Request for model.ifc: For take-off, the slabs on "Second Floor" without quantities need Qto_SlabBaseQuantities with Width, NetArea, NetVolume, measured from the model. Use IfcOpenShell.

First a look at what the model holds.

```python
import ifcopenshell
import ifcopenshell.util.element
import ifcopenshell.util.unit

model = ifcopenshell.open("model.ifc")
print(model.schema)
for unit_type in ("LENGTHUNIT", "AREAUNIT", "VOLUMEUNIT"):
    print(unit_type, ifcopenshell.util.unit.calculate_unit_scale(model, unit_type))
storey = next(s for s in model.by_type("IfcBuildingStorey") if s.Name == "Second Floor")
slabs = [e for e in ifcopenshell.util.element.get_decomposition(storey) if e.is_a("IfcSlab")]
for e in sorted(slabs, key=lambda e: e.id()):
    print(e.id(), e.is_a(), e.Name, list(ifcopenshell.util.element.get_psets(e, qtos_only=True)), sep=" | ")
```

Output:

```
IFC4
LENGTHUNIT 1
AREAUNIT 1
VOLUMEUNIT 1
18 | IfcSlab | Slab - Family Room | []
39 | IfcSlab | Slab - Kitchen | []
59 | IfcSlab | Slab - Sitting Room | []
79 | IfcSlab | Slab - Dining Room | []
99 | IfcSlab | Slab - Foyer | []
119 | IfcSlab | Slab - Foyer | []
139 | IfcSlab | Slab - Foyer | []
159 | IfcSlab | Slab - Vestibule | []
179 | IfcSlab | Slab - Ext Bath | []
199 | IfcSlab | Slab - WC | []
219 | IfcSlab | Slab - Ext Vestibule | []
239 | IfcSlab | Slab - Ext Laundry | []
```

```python
import ifcopenshell
import ifcopenshell.api.pset
import ifcopenshell.geom
import ifcopenshell.util.element
import ifcopenshell.util.shape
import ifcopenshell.util.unit

model = ifcopenshell.open("model.ifc")
unit_scale = ifcopenshell.util.unit.calculate_unit_scale(model)
area_scale = ifcopenshell.util.unit.calculate_unit_scale(model, "AREAUNIT")
volume_scale = ifcopenshell.util.unit.calculate_unit_scale(model, "VOLUMEUNIT")
settings = ifcopenshell.geom.settings()

storey = next(s for s in model.by_type("IfcBuildingStorey") if s.Name == "Second Floor")
slabs = [e for e in ifcopenshell.util.element.get_decomposition(storey) if e.is_a("IfcSlab")]

for e in sorted(slabs, key=lambda e: e.id()):
    if ifcopenshell.util.element.get_psets(e, qtos_only=True, should_inherit=False):
        continue
    # Geometry comes back in metres, in the element's own axes.
    shape = ifcopenshell.geom.create_shape(settings, e)
    values = {
        "Width": ifcopenshell.util.shape.get_z(shape.geometry) / unit_scale,
        "NetArea": ifcopenshell.util.shape.get_footprint_area(shape.geometry) / area_scale,
        "NetVolume": ifcopenshell.util.shape.get_volume(shape.geometry) / volume_scale,
    }
    qto = ifcopenshell.api.pset.add_qto(model, product=e, name="Qto_SlabBaseQuantities")
    ifcopenshell.api.pset.edit_qto(model, qto=qto, properties=values)
    print(e.id(), {k: round(v, 3) for k, v in values.items()})

model.write("model-out.ifc")
```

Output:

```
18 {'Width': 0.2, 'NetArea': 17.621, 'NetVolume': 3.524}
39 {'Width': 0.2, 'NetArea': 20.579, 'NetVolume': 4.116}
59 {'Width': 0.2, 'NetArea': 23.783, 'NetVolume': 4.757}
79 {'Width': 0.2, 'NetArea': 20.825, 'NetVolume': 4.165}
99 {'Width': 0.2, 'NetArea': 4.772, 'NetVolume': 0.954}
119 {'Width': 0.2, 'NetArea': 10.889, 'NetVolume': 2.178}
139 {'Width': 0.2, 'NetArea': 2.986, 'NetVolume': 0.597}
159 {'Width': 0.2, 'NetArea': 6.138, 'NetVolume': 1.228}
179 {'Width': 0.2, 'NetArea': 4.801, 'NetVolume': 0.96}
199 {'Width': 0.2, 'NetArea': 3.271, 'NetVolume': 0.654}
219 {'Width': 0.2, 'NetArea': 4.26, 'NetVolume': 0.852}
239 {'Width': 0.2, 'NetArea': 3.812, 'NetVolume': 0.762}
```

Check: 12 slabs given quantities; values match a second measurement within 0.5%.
